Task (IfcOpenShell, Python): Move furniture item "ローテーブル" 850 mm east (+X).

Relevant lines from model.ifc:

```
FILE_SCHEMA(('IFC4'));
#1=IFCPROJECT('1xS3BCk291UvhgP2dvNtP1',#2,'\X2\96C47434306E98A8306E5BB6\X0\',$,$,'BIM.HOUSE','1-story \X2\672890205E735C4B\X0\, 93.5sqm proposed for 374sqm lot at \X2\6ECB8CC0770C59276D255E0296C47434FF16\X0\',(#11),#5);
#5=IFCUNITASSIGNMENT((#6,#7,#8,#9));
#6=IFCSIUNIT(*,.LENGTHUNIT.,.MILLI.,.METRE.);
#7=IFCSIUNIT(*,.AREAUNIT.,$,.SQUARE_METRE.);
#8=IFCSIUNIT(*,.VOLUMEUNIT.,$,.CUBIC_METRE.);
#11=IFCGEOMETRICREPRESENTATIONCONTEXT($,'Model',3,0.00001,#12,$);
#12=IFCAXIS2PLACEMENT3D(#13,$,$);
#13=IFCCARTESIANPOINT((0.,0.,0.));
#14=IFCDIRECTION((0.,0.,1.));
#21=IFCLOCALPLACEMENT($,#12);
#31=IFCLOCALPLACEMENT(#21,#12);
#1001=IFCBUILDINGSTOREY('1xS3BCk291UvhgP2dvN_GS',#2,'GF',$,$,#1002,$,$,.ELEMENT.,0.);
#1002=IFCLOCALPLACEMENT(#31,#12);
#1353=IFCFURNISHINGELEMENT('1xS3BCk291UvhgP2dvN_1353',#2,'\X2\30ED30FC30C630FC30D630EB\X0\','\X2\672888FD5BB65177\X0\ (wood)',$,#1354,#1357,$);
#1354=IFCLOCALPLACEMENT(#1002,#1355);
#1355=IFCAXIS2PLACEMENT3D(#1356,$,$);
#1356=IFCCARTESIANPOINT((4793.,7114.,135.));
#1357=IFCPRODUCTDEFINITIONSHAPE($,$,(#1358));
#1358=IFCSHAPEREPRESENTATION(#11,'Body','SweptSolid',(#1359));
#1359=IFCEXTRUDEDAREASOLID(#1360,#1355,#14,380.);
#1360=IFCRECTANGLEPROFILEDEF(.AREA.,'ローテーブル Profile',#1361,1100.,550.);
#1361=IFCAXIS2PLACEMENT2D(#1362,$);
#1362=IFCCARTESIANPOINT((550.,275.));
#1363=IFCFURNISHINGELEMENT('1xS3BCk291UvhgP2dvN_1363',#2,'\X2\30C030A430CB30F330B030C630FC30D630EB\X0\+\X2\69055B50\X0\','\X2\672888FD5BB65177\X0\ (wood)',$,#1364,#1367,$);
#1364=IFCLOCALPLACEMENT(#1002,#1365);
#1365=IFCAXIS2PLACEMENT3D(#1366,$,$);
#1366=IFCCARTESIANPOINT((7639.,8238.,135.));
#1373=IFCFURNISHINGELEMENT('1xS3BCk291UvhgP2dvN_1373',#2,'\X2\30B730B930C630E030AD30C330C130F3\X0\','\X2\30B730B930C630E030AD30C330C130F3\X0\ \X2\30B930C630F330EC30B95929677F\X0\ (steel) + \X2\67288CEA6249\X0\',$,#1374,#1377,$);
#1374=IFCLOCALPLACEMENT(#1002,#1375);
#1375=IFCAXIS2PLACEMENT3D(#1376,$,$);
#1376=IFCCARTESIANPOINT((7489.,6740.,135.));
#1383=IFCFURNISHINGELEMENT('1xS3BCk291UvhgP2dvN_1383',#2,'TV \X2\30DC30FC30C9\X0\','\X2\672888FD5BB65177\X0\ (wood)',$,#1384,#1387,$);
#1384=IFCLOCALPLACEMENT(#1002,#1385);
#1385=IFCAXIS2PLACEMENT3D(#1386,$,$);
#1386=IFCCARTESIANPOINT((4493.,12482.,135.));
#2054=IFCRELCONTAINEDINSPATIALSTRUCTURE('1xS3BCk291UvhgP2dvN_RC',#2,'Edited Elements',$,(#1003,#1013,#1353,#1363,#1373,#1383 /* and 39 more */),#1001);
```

```python
import ifcopenshell
import ifcopenshell.api.geometry
import ifcopenshell.util.placement

model = ifcopenshell.open("model.ifc")

item = model.by_id(1353)
matrix = ifcopenshell.util.placement.get_local_placement(item.ObjectPlacement)
matrix[0, 3] += 850.0
ifcopenshell.api.geometry.edit_object_placement(model, product=item, matrix=matrix, is_si=False)

print(ifcopenshell.util.placement.get_local_placement(item.ObjectPlacement).round(3) + 0.0)

model.write("model_rev.ifc")
```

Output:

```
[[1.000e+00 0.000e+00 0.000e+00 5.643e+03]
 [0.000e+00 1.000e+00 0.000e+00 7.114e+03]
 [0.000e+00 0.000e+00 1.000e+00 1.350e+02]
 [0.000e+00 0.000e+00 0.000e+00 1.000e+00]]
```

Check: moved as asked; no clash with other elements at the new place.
